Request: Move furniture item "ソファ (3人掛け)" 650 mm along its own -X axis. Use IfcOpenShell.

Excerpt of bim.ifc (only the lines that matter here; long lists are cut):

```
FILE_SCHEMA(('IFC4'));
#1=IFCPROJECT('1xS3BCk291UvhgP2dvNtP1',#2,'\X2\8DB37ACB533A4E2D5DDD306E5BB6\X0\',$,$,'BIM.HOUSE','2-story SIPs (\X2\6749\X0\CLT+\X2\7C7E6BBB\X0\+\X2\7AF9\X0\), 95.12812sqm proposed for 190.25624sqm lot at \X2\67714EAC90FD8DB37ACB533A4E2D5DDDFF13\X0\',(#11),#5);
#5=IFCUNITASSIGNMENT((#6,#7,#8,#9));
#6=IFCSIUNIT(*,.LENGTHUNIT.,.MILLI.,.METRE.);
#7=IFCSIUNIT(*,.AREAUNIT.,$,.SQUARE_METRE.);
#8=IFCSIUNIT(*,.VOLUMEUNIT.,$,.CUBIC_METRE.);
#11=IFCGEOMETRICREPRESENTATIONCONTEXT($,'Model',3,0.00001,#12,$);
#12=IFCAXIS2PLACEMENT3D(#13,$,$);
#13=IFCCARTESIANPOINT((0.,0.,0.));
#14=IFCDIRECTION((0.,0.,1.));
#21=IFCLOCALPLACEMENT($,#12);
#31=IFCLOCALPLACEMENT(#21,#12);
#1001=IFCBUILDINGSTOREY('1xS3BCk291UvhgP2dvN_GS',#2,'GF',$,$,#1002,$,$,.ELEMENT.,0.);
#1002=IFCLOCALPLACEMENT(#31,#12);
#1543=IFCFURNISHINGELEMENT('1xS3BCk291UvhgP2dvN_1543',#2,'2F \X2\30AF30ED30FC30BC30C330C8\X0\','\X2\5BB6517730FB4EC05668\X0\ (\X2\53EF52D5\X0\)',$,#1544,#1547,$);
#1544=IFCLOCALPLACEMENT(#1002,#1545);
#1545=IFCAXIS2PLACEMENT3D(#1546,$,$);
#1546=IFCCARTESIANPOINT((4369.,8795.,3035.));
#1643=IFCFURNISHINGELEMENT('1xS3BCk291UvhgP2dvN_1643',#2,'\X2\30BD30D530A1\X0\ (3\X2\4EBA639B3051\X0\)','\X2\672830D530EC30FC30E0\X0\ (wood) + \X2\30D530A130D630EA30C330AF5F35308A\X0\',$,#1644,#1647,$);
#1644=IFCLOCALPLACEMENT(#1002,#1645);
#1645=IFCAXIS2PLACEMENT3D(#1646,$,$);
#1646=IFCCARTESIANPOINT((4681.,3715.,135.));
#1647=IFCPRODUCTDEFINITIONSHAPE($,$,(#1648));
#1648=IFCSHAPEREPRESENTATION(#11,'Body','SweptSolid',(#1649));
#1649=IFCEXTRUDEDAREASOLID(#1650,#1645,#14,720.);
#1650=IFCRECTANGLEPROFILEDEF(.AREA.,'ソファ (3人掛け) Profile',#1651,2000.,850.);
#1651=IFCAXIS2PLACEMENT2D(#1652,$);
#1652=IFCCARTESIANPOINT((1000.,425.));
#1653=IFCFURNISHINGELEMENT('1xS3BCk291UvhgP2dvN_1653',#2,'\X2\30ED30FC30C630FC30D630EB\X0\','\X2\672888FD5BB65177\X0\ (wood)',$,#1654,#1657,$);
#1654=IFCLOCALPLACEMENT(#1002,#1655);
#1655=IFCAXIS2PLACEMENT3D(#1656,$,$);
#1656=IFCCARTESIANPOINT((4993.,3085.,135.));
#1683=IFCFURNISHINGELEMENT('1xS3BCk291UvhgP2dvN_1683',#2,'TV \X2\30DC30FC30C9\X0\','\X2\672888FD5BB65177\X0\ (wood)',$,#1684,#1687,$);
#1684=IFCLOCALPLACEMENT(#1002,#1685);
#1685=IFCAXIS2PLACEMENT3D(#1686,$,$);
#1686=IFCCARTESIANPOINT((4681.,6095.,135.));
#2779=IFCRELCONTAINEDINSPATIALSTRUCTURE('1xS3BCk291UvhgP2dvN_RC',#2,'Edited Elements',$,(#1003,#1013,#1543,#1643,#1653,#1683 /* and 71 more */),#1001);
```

```python
import ifcopenshell
import ifcopenshell.api.geometry
import ifcopenshell.util.placement

model = ifcopenshell.open("bim.ifc")

item = model.by_guid("1xS3BCk291UvhgP2dvN_1643")
matrix = ifcopenshell.util.placement.get_local_placement(item.ObjectPlacement)
matrix[:3, 3] -= matrix[:3, 0] * 650.0
ifcopenshell.api.geometry.edit_object_placement(model, product=item, matrix=matrix, is_si=False)

print(ifcopenshell.util.placement.get_local_placement(item.ObjectPlacement).round(3) + 0.0)

model.write("bim_edited.ifc")
```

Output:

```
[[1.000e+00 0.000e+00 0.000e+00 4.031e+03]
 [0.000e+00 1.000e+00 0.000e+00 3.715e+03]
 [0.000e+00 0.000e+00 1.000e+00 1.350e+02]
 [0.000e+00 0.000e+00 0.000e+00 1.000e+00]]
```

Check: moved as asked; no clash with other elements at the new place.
